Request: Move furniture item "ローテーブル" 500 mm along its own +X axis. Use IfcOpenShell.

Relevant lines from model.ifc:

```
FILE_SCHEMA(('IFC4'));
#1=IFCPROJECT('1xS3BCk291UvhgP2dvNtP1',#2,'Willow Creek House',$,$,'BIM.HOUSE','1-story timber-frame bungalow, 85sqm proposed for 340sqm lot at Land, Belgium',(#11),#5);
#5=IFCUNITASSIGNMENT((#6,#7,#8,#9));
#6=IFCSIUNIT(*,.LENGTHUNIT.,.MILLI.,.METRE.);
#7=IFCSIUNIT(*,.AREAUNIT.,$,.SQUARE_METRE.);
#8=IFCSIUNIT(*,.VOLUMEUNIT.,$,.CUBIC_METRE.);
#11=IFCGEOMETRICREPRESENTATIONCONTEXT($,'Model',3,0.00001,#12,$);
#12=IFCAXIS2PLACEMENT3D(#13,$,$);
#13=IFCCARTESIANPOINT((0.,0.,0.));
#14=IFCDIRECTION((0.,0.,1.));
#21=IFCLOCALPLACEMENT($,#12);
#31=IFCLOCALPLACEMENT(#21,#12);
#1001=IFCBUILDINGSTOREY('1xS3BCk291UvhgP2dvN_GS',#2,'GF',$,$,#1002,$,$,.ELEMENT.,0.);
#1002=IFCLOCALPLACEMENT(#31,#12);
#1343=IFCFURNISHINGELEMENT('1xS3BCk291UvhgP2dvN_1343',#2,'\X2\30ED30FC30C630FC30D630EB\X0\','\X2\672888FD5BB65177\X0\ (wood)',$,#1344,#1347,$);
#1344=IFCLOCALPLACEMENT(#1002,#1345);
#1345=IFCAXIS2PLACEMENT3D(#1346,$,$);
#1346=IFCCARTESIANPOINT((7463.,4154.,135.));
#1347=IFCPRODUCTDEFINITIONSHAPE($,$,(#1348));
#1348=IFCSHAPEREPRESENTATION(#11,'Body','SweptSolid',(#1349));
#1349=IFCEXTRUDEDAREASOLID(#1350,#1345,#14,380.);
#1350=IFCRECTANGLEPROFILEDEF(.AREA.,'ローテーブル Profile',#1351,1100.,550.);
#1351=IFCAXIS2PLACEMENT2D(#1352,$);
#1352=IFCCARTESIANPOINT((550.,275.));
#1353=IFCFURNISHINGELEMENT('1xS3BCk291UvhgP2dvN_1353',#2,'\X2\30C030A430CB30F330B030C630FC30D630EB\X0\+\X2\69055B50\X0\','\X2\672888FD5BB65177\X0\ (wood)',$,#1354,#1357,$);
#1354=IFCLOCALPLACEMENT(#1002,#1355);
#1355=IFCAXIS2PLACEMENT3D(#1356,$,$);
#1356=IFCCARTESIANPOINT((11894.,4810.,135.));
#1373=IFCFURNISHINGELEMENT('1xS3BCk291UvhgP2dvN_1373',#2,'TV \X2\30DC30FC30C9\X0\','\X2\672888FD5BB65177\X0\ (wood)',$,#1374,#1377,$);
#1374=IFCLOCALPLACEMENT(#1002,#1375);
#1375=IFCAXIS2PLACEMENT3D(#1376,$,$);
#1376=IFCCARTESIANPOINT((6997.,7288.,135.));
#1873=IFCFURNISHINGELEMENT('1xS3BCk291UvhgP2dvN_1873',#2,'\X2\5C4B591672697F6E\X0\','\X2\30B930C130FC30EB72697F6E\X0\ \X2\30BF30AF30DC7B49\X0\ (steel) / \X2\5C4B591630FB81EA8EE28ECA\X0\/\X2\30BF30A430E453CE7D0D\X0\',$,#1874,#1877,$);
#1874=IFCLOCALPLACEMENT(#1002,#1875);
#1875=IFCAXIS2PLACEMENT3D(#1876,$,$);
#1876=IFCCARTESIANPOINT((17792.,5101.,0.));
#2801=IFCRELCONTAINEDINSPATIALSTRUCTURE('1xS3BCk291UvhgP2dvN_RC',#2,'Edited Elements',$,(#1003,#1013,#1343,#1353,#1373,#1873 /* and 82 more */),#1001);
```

```python
import ifcopenshell
import ifcopenshell.api.geometry
import ifcopenshell.util.placement

model = ifcopenshell.open("model.ifc")

item = model.by_id(1343)
matrix = ifcopenshell.util.placement.get_local_placement(item.ObjectPlacement)
matrix[:3, 3] += matrix[:3, 0] * 500.0
ifcopenshell.api.geometry.edit_object_placement(model, product=item, matrix=matrix, is_si=False)

print(ifcopenshell.util.placement.get_local_placement(item.ObjectPlacement).round(3) + 0.0)

model.write("model_rev.ifc")
```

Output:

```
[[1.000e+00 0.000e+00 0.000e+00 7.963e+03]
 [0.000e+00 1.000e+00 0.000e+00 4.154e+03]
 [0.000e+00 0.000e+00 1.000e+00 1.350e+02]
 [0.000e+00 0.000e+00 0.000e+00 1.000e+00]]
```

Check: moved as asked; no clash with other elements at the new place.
